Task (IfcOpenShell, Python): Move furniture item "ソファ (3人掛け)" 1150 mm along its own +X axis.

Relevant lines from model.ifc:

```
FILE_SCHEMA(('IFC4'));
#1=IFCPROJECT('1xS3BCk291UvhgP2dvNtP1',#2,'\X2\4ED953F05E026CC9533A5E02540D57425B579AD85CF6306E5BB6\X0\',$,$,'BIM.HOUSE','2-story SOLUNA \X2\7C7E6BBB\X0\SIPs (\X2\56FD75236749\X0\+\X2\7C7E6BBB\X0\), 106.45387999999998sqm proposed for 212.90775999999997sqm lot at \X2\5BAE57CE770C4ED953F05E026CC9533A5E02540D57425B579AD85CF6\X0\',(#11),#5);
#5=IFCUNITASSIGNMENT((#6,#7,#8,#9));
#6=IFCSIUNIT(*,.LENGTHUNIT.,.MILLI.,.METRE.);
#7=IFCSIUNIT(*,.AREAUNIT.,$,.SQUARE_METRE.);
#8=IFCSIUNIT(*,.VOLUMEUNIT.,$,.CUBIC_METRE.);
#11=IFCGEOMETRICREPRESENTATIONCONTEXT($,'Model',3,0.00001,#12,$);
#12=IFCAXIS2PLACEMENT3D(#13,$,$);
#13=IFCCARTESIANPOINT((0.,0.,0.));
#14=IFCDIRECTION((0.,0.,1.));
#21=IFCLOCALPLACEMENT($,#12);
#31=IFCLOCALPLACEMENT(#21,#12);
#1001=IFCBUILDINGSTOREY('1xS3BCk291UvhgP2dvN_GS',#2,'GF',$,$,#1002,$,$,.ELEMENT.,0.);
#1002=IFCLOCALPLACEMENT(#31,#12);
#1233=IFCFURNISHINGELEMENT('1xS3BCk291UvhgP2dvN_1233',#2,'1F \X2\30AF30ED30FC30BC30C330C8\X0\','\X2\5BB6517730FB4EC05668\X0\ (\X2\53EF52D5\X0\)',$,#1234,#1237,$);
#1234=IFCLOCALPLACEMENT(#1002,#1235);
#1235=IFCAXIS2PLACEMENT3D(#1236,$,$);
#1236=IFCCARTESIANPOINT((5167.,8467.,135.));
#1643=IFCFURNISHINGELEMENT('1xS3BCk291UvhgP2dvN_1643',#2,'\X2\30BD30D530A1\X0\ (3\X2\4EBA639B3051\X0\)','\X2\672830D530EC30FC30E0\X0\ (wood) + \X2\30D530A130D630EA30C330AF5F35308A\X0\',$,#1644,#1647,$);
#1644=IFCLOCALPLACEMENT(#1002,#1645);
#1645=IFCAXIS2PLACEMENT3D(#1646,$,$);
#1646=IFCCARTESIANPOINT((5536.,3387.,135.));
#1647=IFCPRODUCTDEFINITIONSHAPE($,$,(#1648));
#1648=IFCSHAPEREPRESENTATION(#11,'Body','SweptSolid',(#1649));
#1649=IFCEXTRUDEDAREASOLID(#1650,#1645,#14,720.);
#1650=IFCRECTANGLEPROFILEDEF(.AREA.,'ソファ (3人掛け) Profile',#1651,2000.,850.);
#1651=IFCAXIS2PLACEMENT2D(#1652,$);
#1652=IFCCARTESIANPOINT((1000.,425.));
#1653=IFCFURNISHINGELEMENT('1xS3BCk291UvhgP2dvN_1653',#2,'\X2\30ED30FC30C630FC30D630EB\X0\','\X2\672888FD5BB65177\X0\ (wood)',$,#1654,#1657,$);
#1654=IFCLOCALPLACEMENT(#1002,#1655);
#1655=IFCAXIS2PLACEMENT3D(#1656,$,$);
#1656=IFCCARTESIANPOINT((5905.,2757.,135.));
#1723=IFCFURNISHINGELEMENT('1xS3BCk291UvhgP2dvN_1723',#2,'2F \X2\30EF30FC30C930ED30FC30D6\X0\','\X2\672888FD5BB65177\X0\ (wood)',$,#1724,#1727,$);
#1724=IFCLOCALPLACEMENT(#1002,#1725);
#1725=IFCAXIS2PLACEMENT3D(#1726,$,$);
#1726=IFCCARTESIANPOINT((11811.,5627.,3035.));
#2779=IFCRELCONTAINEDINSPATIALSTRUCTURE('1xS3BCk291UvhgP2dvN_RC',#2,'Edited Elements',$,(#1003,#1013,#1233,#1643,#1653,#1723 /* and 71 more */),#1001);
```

```python
import ifcopenshell
import ifcopenshell.api.geometry
import ifcopenshell.util.placement
import ifcopenshell.util.unit

model = ifcopenshell.open("model.ifc")
unit_scale = ifcopenshell.util.unit.calculate_unit_scale(model)

item = model.by_guid("1xS3BCk291UvhgP2dvN_1643")
matrix = ifcopenshell.util.placement.get_local_placement(item.ObjectPlacement)
matrix[:3, 3] += matrix[:3, 0] * 1.15 / unit_scale
ifcopenshell.api.geometry.edit_object_placement(model, product=item, matrix=matrix, is_si=False)

print(ifcopenshell.util.placement.get_local_placement(item.ObjectPlacement).round(3) + 0.0)

model.write("model_edited.ifc")
```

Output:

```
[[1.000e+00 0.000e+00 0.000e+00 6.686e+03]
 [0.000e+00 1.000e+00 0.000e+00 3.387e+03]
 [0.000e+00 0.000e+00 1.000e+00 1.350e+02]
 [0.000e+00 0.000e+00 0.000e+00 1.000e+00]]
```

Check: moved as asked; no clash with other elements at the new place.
